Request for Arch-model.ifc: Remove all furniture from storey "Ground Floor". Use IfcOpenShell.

First a look at what the model holds.

```python
import ifcopenshell
import ifcopenshell.util.element

model = ifcopenshell.open("Arch-model.ifc")
print(model.schema)
storey = next(s for s in model.by_type("IfcBuildingStorey") if s.Name == "Ground Floor")
furniture = [e for e in ifcopenshell.util.element.get_decomposition(storey) if e.is_a("IfcFurnishingElement")]
seen = {}
for e in furniture:
    element_type = ifcopenshell.util.element.get_type(e)
    name = element_type.Name if element_type not in (None, e) else None
    seen[name] = seen.get(name, 0) + 1
for name, count in sorted(seen.items(), key=str):
    print(count, "x", name)
```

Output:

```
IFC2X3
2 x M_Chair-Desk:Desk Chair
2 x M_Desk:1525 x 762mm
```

```python
import ifcopenshell
import ifcopenshell.api.root
import ifcopenshell.util.element

model = ifcopenshell.open("Arch-model.ifc")

storey = next(s for s in model.by_type("IfcBuildingStorey") if s.Name == "Ground Floor")
furniture = [e for e in ifcopenshell.util.element.get_decomposition(storey) if e.is_a("IfcFurnishingElement")]

for e in furniture:
    ifcopenshell.api.root.remove_product(model, product=e)
print(len(furniture), "removed")

model.write("Arch-model_updated.ifc")
```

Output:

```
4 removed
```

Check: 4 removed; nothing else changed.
